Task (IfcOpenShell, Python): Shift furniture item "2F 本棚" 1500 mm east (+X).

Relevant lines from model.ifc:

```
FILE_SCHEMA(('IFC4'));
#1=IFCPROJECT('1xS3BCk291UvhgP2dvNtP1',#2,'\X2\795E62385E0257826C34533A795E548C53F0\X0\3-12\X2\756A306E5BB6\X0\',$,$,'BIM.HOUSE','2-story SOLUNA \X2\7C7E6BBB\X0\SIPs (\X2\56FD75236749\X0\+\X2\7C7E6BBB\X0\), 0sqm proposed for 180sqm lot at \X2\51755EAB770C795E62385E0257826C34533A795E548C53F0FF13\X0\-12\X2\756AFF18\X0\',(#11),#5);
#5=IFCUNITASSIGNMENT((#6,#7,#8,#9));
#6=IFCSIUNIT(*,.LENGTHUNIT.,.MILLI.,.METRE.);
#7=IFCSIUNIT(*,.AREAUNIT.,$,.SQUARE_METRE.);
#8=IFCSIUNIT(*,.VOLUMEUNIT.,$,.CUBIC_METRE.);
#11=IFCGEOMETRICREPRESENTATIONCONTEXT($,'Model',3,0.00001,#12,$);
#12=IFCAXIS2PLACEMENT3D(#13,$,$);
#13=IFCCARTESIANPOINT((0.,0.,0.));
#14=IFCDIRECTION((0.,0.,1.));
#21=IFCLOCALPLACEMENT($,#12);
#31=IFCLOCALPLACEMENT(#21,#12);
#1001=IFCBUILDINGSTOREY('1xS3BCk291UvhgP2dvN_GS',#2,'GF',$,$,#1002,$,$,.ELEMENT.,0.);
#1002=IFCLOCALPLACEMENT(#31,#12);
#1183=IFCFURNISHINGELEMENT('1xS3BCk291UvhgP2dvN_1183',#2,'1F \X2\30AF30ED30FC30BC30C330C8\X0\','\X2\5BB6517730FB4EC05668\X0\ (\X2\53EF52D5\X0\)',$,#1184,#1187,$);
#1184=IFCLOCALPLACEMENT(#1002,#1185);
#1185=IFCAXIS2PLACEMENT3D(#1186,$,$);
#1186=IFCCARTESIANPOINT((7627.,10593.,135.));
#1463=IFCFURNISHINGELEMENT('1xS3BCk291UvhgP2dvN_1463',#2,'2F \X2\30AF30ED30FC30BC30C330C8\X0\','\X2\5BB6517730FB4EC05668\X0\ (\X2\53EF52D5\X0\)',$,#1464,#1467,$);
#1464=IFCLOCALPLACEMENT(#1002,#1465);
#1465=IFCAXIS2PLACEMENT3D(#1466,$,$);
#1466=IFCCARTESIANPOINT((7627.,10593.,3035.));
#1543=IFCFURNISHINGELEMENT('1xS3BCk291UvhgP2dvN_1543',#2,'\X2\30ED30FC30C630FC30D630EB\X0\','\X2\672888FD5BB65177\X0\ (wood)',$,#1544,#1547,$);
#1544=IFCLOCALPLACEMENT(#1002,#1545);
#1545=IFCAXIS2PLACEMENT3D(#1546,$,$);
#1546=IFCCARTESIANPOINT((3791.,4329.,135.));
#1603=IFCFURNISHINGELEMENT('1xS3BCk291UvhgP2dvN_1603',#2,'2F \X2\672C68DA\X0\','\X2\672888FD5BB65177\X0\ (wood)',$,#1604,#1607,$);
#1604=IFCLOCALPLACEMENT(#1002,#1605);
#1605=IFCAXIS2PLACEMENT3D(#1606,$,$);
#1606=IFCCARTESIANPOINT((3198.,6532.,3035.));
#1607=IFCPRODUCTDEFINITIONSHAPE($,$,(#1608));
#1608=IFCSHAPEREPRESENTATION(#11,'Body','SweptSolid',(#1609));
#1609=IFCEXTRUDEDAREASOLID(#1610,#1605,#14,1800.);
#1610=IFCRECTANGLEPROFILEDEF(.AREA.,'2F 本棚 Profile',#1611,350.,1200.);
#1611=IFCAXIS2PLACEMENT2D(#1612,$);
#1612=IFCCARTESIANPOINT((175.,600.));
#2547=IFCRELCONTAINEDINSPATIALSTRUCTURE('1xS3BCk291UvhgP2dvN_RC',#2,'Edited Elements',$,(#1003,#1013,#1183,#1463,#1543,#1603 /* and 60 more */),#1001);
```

```python
import ifcopenshell
import ifcopenshell.api.geometry
import ifcopenshell.util.placement
import ifcopenshell.util.unit

model = ifcopenshell.open("model.ifc")
unit_scale = ifcopenshell.util.unit.calculate_unit_scale(model)

item = model.by_guid("1xS3BCk291UvhgP2dvN_1603")
matrix = ifcopenshell.util.placement.get_local_placement(item.ObjectPlacement)
matrix[0, 3] += 1.5 / unit_scale
ifcopenshell.api.geometry.edit_object_placement(model, product=item, matrix=matrix, is_si=False)

print(ifcopenshell.util.placement.get_local_placement(item.ObjectPlacement).round(3) + 0.0)

model.write("model_edited.ifc")
```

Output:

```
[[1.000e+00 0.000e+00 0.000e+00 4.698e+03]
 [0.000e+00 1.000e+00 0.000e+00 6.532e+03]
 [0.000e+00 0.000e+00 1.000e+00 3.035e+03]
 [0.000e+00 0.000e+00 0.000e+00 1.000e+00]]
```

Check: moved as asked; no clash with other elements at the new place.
